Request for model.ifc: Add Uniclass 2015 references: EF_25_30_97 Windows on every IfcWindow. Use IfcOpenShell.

First a look at what the model holds.

```python
import ifcopenshell

model = ifcopenshell.open("model.ifc")
print(model.schema)
print("classifications:", [c.Name for c in model.by_type("IfcClassification")])
for ifc_class in ("IfcDoor", "IfcRoof", "IfcStair", "IfcWall", "IfcWindow"):
    print(ifc_class, len(model.by_type(ifc_class)))
```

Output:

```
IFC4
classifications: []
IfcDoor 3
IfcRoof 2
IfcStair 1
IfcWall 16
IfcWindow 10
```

```python
import ifcopenshell
import ifcopenshell.api.classification

model = ifcopenshell.open("model.ifc")

system = ifcopenshell.api.classification.add_classification(model, classification="Uniclass 2015")

codes = {
    "IfcWindow": ("EF_25_30_97", "Windows"),
}
for ifc_class, (code, name) in codes.items():
    products = model.by_type(ifc_class)
    ifcopenshell.api.classification.add_reference(
        model, products=products, classification=system, identification=code, name=name
    )
    print(code, len(products))

model.write("model_updated.ifc")
```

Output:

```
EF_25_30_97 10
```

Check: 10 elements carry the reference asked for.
